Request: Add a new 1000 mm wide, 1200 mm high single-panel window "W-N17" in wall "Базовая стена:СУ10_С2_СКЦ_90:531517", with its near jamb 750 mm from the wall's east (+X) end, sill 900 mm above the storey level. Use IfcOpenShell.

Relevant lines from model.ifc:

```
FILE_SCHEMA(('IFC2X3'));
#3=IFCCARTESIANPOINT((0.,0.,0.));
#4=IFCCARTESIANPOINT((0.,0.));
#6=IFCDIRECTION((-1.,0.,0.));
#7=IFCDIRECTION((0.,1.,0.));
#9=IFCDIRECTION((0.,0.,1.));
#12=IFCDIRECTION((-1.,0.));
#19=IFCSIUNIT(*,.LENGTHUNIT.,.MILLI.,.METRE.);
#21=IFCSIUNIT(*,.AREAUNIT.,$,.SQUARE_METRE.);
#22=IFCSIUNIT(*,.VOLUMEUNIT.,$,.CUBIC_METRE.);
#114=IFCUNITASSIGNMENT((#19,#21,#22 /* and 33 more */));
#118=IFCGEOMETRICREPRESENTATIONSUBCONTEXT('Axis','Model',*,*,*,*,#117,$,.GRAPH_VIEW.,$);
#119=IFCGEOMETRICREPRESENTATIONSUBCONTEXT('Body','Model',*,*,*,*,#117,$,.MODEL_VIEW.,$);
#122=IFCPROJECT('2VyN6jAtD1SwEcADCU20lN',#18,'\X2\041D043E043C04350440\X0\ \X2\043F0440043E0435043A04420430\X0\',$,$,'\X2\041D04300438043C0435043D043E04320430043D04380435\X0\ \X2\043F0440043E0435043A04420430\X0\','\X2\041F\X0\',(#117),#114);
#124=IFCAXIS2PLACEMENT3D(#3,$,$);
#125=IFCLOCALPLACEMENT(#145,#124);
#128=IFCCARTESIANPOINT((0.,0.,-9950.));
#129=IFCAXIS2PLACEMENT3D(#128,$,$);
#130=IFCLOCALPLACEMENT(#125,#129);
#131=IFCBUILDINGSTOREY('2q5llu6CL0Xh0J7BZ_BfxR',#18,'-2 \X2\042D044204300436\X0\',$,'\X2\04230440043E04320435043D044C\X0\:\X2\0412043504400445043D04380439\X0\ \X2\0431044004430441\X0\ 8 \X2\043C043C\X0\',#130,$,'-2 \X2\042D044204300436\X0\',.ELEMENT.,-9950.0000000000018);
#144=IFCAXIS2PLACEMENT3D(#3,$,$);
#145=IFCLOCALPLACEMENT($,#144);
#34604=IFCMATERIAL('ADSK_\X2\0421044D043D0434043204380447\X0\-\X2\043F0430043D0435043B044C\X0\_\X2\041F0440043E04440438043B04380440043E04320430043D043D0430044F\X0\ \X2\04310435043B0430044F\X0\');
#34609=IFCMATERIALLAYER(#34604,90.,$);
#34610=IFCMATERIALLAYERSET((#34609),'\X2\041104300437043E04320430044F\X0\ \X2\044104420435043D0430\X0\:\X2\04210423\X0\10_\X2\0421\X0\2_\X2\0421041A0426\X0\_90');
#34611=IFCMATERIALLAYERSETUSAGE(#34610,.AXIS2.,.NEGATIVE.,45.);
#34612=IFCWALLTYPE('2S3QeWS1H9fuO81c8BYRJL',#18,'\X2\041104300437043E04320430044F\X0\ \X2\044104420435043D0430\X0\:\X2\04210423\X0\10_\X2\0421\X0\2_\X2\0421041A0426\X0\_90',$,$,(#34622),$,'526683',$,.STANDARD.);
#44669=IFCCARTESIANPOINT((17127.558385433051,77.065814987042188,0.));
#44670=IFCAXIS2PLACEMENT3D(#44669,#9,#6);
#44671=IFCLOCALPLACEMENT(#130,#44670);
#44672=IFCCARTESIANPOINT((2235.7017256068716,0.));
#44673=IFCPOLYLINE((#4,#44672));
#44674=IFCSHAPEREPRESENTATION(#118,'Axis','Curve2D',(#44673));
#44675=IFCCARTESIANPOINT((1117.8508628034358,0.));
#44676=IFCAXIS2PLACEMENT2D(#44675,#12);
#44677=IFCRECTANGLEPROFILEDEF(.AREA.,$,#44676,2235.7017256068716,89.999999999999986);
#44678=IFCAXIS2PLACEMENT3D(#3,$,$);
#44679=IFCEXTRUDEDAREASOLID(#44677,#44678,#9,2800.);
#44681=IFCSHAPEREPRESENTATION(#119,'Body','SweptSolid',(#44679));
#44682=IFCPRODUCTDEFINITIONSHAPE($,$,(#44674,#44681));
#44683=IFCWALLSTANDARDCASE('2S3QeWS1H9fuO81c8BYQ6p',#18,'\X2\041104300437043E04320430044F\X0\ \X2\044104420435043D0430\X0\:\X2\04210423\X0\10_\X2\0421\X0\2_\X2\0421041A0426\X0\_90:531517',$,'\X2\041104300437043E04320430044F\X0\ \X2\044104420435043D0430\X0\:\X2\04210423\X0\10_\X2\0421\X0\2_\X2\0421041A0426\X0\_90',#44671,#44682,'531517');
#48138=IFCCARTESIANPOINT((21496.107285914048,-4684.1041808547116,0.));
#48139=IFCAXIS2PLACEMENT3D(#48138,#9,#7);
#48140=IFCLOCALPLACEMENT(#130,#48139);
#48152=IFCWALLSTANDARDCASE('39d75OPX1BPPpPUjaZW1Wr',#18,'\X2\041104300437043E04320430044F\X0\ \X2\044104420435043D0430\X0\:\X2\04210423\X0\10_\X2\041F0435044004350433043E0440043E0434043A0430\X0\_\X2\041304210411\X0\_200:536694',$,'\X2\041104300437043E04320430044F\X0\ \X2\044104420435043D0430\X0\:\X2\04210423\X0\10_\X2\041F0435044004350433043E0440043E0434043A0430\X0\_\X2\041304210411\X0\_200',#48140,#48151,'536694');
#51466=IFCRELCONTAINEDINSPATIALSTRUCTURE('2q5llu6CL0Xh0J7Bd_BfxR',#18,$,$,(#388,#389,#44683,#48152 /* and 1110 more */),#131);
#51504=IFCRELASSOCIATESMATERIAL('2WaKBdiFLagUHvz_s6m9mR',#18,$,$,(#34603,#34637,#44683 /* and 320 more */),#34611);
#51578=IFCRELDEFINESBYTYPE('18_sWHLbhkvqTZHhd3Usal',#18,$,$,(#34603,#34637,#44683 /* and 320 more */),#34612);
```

```python
import numpy as np
import ifcopenshell
import ifcopenshell.api.feature
import ifcopenshell.api.geometry
import ifcopenshell.api.root
import ifcopenshell.api.spatial
import ifcopenshell.api.type
import ifcopenshell.geom
import ifcopenshell.util.element
import ifcopenshell.util.placement
import ifcopenshell.util.representation
import ifcopenshell.util.shape
import ifcopenshell.util.unit

model = ifcopenshell.open("model.ifc")
unit_scale = ifcopenshell.util.unit.calculate_unit_scale(model)
settings = ifcopenshell.geom.settings()


def volume(element):
    """Net volume in cubic metres, openings subtracted."""
    shape = ifcopenshell.geom.create_shape(settings, element)
    return ifcopenshell.util.shape.get_volume(shape.geometry)


wall = model.by_guid("2S3QeWS1H9fuO81c8BYQ6p")
storey = ifcopenshell.util.element.get_container(wall, ifc_class="IfcBuildingStorey")
context = ifcopenshell.util.representation.get_context(model, "Model", "Body", "MODEL_VIEW")
before = volume(wall)

width, height, from_end, sill = 1, 1.2, 0.75, 0.9  # metres

# The wall runs along its own X axis, and the end named is its -X end.
wall_shape = ifcopenshell.geom.create_shape(settings, wall)
x, y, z = ifcopenshell.util.shape.get_vertices(wall_shape.geometry).T
start = x.min() + from_end
face, thickness = float(y.min()), float(y.max() - y.min())
wall_matrix = ifcopenshell.util.placement.get_local_placement(wall.ObjectPlacement)
level = ifcopenshell.util.placement.get_local_placement(storey.ObjectPlacement)[2, 3]


def in_wall(x, y):
    """Placement at x, y metres in the wall's axes, at sill height."""
    matrix = wall_matrix.copy()
    matrix[:, 3] = wall_matrix @ np.array([x / unit_scale, y / unit_scale, 0.0, 1.0])
    matrix[2, 3] = level + sill / unit_scale
    return matrix


# Opening: a box that overshoots both wall faces by 50 mm.
opening = ifcopenshell.api.root.create_entity(model, ifc_class="IfcOpeningElement")
box = ifcopenshell.api.geometry.add_wall_representation(
    model, context=context, length=width, height=height, thickness=thickness + 0.1
)
ifcopenshell.api.geometry.assign_representation(model, product=opening, representation=box)
ifcopenshell.api.geometry.edit_object_placement(model, product=opening, matrix=in_wall(start, face - 0.05), is_si=False)
ifcopenshell.api.feature.add_feature(model, feature=opening, element=wall)

window = ifcopenshell.api.root.create_entity(model, ifc_class="IfcWindow", name="W-N17")
window.OverallWidth, window.OverallHeight = width / unit_scale, height / unit_scale
body = ifcopenshell.api.geometry.add_window_representation(
    model,
    context=context,
    overall_width=window.OverallWidth,
    overall_height=window.OverallHeight,
    partition_type="SINGLE_PANEL",
)
ifcopenshell.api.geometry.assign_representation(model, product=window, representation=body)
ifcopenshell.api.spatial.assign_container(model, products=[window], relating_structure=storey)
fills = ifcopenshell.api.feature.add_filling(model, opening=opening, element=window)
fills.OwnerHistory = window.OwnerHistory  # required in IFC2X3

# IFC2X3 keeps the operation on the window style.
style = ifcopenshell.api.root.create_entity(model, ifc_class="IfcWindowStyle", name="W-N17")
style.OperationType, style.ConstructionType = "SINGLE_PANEL", "NOTDEFINED"
style.ParameterTakesPrecedence = style.Sizeable = False
ifcopenshell.api.type.assign_type(model, related_objects=[window], relating_type=style)

# Centre the window in the wall's thickness.
ifcopenshell.api.geometry.edit_object_placement(model, product=window, matrix=in_wall(start, face), is_si=False)
window_shape = ifcopenshell.geom.create_shape(settings, window)
depth = ifcopenshell.util.shape.get_vertices(window_shape.geometry)[:, 1]
offset = face + thickness / 2 - (depth.min() + depth.max()) / 2
ifcopenshell.api.geometry.edit_object_placement(model, product=window, matrix=in_wall(start, offset), is_si=False)

after = volume(wall)

print(f"wall volume {before:.3f} -> {after:.3f} m3")

model.write("model_edited.ifc")
```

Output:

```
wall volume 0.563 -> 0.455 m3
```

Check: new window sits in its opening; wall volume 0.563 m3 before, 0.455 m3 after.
